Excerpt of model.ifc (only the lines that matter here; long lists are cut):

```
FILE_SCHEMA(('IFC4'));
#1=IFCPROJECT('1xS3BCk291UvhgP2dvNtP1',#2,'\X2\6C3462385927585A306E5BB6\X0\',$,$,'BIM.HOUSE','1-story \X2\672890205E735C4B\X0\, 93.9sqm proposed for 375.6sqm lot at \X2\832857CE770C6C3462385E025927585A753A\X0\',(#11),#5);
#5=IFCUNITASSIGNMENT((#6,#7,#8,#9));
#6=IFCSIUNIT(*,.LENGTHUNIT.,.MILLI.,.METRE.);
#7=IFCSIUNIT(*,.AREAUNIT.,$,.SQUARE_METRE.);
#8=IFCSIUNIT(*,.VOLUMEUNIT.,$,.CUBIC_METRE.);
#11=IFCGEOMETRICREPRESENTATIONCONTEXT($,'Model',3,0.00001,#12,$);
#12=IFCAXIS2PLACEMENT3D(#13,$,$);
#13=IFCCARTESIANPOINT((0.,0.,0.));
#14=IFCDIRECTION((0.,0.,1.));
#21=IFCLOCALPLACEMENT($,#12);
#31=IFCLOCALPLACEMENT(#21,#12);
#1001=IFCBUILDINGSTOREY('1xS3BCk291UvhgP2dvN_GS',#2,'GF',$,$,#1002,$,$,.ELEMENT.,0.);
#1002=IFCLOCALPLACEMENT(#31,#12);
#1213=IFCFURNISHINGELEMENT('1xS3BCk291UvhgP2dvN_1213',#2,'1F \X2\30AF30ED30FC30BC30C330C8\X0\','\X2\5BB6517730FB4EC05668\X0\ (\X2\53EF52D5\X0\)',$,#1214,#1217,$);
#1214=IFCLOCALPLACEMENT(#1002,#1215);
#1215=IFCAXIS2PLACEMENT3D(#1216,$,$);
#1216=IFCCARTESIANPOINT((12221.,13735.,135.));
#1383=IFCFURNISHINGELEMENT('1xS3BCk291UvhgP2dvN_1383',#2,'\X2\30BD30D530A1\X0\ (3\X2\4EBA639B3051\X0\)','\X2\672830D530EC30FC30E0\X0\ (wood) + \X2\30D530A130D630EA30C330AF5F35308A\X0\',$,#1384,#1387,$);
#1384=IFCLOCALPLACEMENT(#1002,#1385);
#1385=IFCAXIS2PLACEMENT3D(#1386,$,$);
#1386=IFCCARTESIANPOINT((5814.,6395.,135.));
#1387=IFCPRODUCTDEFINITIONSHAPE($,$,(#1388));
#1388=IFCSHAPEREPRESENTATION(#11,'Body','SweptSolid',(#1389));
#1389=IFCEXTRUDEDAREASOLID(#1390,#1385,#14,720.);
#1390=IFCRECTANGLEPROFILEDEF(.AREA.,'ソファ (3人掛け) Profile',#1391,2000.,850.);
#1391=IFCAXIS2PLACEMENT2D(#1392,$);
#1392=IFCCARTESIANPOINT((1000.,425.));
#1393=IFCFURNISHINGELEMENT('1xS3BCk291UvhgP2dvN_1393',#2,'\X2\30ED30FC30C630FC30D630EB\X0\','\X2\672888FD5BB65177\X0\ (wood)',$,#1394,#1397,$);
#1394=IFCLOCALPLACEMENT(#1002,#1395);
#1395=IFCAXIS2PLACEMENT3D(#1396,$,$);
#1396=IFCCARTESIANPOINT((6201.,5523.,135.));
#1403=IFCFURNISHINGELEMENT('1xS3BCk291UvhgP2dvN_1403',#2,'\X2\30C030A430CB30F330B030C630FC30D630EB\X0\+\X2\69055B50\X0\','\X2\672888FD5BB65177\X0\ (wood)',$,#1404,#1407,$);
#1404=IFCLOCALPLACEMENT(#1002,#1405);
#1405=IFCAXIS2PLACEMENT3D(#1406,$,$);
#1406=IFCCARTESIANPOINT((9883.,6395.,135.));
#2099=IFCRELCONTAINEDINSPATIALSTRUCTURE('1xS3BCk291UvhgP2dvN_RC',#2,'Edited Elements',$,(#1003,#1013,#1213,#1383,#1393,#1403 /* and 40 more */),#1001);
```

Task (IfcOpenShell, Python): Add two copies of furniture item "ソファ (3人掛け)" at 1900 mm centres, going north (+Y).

```python
import numpy as np
import ifcopenshell
import ifcopenshell.api.geometry
import ifcopenshell.api.root
import ifcopenshell.util.element
import ifcopenshell.util.placement

model = ifcopenshell.open("model.ifc")


def reuse_history(source, copy):
    """copy_class also copies each property set's owner history, people and application; keep the originals."""
    for rel in copy.IsDefinedBy:
        if rel.is_a("IfcRelDefinesByProperties") and (history := rel.RelatingPropertyDefinition.OwnerHistory):
            rel.RelatingPropertyDefinition.OwnerHistory = source.OwnerHistory
            ifcopenshell.util.element.remove_deep2(model, history)


source = model.by_guid("1xS3BCk291UvhgP2dvN_1383")
base = ifcopenshell.util.placement.get_local_placement(source.ObjectPlacement)
step = np.array([0.0, 1.0, 0.0]) * 1900.0

for i in range(1, 3):
    copy = ifcopenshell.api.root.copy_class(model, product=source)
    copy.Representation = ifcopenshell.util.element.copy_deep(
        model, source.Representation, exclude=["IfcGeometricRepresentationContext", "IfcRepresentationMap"]
    )
    reuse_history(source, copy)
    matrix = base.copy()
    matrix[:3, 3] += i * step
    print("added at", matrix[:3, 3].round(3) + 0.0)
    ifcopenshell.api.geometry.edit_object_placement(model, product=copy, matrix=matrix, is_si=False)

model.write("model-out.ifc")
```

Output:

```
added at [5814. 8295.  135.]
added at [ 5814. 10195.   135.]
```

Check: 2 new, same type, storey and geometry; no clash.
